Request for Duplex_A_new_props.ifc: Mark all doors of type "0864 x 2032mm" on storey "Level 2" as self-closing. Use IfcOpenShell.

First a look at what the model holds.

```python
import ifcopenshell
import ifcopenshell.util.element

model = ifcopenshell.open("Duplex_A_new_props.ifc")
print(model.schema)
storey = next(s for s in model.by_type("IfcBuildingStorey") if s.Name == "Level 2")
doors = [e for e in ifcopenshell.util.element.get_decomposition(storey) if e.is_a("IfcDoor")]
seen = {}
for e in doors:
    element_type = ifcopenshell.util.element.get_type(e)
    key = (element_type.Name if element_type != e and element_type else None, ifcopenshell.util.element.get_pset(e, "Pset_DoorCommon", "SelfClosing"))
    seen[key] = seen.get(key, 0) + 1
for (name, value), count in sorted(seen.items(), key=str):
    print(count, "x", name, "|", value)
```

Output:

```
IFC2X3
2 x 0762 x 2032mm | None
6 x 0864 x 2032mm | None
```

```python
import ifcopenshell
import ifcopenshell.api.pset
import ifcopenshell.util.element

model = ifcopenshell.open("Duplex_A_new_props.ifc")

storey = next(s for s in model.by_type("IfcBuildingStorey") if s.Name == "Level 2")
doors = [e for e in ifcopenshell.util.element.get_decomposition(storey) if e.is_a("IfcDoor")]

count = 0
for e in doors:
    element_type = ifcopenshell.util.element.get_type(e)
    if element_type in (None, e) or element_type.Name != "0864 x 2032mm":
        continue
    # add_pset returns the element's existing set when there is one.
    pset = ifcopenshell.api.pset.add_pset(model, product=e, name="Pset_DoorCommon")
    ifcopenshell.api.pset.edit_pset(model, pset=pset, properties={"SelfClosing": True})
    count += 1

print(count, "doors updated")

model.write("Duplex_A_new_props_edited.ifc")
```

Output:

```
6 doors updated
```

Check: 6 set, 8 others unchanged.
